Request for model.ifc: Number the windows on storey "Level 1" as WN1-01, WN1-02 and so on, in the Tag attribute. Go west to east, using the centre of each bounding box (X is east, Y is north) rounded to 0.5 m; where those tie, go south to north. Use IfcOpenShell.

First a look at what the model holds.

```python
import ifcopenshell
import ifcopenshell.util.element
import ifcopenshell.util.placement

model = ifcopenshell.open("model.ifc")
print(model.schema)
storey = next(s for s in model.by_type("IfcBuildingStorey") if s.Name == "Level 1")
windows = [e for e in ifcopenshell.util.element.get_decomposition(storey) if e.is_a("IfcWindow")]
for e in sorted(windows, key=lambda e: e.id()):
    origin = ifcopenshell.util.placement.get_local_placement(e.ObjectPlacement)[:3, 3]
    print(e.id(), e.Tag, e.Name, origin.round(2) + 0.0, sep=" | ")
```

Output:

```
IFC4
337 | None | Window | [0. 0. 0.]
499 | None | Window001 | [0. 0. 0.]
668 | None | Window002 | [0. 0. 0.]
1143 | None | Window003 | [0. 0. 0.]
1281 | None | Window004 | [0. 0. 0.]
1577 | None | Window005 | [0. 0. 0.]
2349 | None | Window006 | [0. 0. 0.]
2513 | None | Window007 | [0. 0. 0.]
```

```python
import ifcopenshell
import ifcopenshell.geom
import ifcopenshell.util.element
import ifcopenshell.util.shape

model = ifcopenshell.open("model.ifc")
settings = ifcopenshell.geom.settings()
settings.set("use-world-coords", True)


def centre(element):
    shape = ifcopenshell.geom.create_shape(settings, element)
    return ifcopenshell.util.shape.get_bbox_centroid(shape.geometry)


storey = next(s for s in model.by_type("IfcBuildingStorey") if s.Name == "Level 1")
windows = [e for e in ifcopenshell.util.element.get_decomposition(storey) if e.is_a("IfcWindow")]

# Insertion points can sit at a corner or the storey origin, so sort by the geometry (in metres).
centres = {e: centre(e) for e in windows}
windows.sort(key=lambda e: (round(centres[e][0] / 0.5), centres[e][1]))

for i, e in enumerate(windows, start=1):
    number = f"WN1-{i:02d}"
    e.Tag = number
    print(e.id(), number)

model.write("model_updated.ifc")
```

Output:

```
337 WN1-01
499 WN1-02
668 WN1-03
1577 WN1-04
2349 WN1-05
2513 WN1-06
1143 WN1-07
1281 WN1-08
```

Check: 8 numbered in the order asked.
